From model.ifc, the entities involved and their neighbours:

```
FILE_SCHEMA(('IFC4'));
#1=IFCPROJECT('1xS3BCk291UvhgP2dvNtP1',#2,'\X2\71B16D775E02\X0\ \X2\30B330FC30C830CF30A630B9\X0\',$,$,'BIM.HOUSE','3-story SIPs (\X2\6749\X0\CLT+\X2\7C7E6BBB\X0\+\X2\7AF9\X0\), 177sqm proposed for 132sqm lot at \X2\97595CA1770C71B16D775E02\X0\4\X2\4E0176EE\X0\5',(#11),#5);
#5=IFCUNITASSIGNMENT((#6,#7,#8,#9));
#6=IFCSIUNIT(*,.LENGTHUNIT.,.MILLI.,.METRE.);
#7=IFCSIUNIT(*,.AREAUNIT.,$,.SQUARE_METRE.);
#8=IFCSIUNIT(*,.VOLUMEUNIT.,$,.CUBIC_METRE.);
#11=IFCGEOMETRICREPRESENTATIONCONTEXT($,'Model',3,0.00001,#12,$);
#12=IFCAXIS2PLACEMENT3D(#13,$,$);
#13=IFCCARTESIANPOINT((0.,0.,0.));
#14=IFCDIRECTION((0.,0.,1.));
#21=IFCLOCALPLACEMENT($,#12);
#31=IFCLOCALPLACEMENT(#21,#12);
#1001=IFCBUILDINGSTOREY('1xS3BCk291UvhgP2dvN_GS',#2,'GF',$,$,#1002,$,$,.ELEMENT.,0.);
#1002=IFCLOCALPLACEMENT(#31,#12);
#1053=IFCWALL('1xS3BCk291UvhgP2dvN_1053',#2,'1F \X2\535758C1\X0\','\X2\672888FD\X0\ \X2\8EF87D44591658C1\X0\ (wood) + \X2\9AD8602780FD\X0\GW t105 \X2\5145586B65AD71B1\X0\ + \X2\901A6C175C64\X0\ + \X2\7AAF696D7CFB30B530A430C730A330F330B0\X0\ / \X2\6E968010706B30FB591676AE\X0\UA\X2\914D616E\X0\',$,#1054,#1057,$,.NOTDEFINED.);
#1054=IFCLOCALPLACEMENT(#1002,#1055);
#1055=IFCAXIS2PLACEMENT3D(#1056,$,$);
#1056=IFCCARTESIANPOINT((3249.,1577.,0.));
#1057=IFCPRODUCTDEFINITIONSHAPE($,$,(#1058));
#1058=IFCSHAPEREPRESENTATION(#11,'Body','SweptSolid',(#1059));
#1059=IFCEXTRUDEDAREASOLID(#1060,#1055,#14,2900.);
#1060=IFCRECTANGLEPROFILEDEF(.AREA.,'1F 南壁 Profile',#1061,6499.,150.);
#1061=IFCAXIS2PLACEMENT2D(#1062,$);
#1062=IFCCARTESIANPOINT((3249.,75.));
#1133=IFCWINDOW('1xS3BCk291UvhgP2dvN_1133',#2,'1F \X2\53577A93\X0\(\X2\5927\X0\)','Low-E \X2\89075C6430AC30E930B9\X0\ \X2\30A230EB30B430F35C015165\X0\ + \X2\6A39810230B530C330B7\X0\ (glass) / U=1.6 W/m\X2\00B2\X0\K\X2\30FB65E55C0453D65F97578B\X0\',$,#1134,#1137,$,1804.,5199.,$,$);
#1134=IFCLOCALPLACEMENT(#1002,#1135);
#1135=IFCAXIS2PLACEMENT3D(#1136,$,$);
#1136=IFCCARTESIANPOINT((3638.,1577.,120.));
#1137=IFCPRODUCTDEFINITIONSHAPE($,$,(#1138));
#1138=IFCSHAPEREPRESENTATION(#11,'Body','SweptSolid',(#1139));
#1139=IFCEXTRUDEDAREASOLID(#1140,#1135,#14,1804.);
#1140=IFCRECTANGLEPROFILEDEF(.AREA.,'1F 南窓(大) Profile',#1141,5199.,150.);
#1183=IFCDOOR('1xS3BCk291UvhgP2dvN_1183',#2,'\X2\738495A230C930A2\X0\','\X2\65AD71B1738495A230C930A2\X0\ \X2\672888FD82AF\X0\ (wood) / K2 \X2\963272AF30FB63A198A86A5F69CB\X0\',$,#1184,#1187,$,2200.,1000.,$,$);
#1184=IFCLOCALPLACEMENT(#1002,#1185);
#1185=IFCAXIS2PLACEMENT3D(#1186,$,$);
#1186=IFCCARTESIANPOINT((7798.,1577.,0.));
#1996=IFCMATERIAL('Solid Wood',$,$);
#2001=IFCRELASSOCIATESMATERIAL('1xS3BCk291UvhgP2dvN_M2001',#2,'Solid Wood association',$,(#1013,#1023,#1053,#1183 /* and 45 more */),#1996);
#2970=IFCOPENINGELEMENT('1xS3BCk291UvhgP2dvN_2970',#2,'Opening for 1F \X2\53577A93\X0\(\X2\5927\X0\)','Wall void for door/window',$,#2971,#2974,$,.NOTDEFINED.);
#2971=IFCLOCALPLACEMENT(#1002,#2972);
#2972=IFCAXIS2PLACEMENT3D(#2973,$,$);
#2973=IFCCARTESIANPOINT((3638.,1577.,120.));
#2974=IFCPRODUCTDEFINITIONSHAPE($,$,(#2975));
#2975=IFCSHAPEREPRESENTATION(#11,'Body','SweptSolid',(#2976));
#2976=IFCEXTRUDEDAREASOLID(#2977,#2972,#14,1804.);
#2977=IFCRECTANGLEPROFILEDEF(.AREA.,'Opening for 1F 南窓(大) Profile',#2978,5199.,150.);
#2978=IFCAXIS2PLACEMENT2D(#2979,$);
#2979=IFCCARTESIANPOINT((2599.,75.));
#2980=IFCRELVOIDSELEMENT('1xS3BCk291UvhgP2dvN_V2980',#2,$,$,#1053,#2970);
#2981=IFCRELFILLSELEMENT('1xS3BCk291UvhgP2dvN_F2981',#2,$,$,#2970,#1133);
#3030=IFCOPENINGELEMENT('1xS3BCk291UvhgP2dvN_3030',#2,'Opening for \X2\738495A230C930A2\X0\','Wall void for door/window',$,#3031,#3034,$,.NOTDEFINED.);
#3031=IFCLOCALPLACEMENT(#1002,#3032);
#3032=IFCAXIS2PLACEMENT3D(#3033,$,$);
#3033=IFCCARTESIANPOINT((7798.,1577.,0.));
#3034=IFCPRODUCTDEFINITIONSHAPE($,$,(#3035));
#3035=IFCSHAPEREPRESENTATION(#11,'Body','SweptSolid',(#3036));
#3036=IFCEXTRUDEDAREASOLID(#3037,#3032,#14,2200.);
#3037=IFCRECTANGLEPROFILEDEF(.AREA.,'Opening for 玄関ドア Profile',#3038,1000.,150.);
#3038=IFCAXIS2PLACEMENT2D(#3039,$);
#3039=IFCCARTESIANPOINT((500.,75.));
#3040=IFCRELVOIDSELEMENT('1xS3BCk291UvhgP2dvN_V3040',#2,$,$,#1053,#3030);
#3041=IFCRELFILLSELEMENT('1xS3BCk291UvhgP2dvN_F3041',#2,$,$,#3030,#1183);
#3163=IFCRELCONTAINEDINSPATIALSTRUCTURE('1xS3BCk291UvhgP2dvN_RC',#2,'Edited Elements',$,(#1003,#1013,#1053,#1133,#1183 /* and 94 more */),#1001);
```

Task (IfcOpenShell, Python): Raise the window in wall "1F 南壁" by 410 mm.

```python
import numpy as np
import ifcopenshell
import ifcopenshell.api.geometry
import ifcopenshell.util.placement
import ifcopenshell.util.unit

model = ifcopenshell.open("model.ifc")
unit_scale = ifcopenshell.util.unit.calculate_unit_scale(model)

window = model.by_id(1133)
opening = window.FillsVoids[0].RelatingOpeningElement
dz = 410.0

shift = np.array([0.0, 0.0, dz])
# The window is not placed relative to its opening, so move both.
for product in (opening, window):
    matrix = ifcopenshell.util.placement.get_local_placement(product.ObjectPlacement)
    matrix[:3, 3] += shift
    ifcopenshell.api.geometry.edit_object_placement(model, product=product, matrix=matrix, is_si=False)

print(f"moved by {dz * unit_scale:+.3f} m")

model.write("model-out.ifc")
```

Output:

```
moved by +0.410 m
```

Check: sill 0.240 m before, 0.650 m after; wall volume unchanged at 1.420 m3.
